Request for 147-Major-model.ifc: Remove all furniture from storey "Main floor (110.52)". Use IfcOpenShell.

First a look at what the model holds.

```python
import ifcopenshell
import ifcopenshell.util.element

model = ifcopenshell.open("147-Major-model.ifc")
print(model.schema)
storey = next(s for s in model.by_type("IfcBuildingStorey") if s.Name == "Main floor (110.52)")
furniture = [e for e in ifcopenshell.util.element.get_decomposition(storey) if e.is_a("IfcFurnishingElement")]
seen = {}
for e in furniture:
    element_type = ifcopenshell.util.element.get_type(e)
    name = element_type.Name if element_type not in (None, e) else None
    seen[name] = seen.get(name, 0) + 1
for name, count in sorted(seen.items(), key=str):
    print(count, "x", name)
```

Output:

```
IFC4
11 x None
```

```python
import ifcopenshell
import ifcopenshell.api.root
import ifcopenshell.util.element

model = ifcopenshell.open("147-Major-model.ifc")

storey = next(s for s in model.by_type("IfcBuildingStorey") if s.Name == "Main floor (110.52)")
furniture = [e for e in ifcopenshell.util.element.get_decomposition(storey) if e.is_a("IfcFurnishingElement")]

for e in furniture:
    ifcopenshell.api.root.remove_product(model, product=e)
print(len(furniture), "removed")

model.write("147-Major-model_rev.ifc")
```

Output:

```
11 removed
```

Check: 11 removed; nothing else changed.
